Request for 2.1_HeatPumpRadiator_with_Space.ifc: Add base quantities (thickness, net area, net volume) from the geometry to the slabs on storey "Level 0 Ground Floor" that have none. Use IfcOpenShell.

First a look at what the model holds.

```python
import ifcopenshell
import ifcopenshell.util.element
import ifcopenshell.util.unit

model = ifcopenshell.open("2.1_HeatPumpRadiator_with_Space.ifc")
print(model.schema)
for unit_type in ("LENGTHUNIT", "AREAUNIT", "VOLUMEUNIT"):
    print(unit_type, ifcopenshell.util.unit.calculate_unit_scale(model, unit_type))
storey = next(s for s in model.by_type("IfcBuildingStorey") if s.Name == "Level 0 Ground Floor")
slabs = [e for e in ifcopenshell.util.element.get_decomposition(storey) if e.is_a("IfcSlab")]
for e in sorted(slabs, key=lambda e: e.id()):
    print(e.id(), e.is_a(), e.Name, list(ifcopenshell.util.element.get_psets(e, qtos_only=True)), sep=" | ")
```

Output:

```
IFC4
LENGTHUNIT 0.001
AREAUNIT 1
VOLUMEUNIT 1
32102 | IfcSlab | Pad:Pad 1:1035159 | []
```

```python
import ifcopenshell
import ifcopenshell.api.pset
import ifcopenshell.geom
import ifcopenshell.util.element
import ifcopenshell.util.shape
import ifcopenshell.util.unit

model = ifcopenshell.open("2.1_HeatPumpRadiator_with_Space.ifc")
unit_scale = ifcopenshell.util.unit.calculate_unit_scale(model)
area_scale = ifcopenshell.util.unit.calculate_unit_scale(model, "AREAUNIT")
volume_scale = ifcopenshell.util.unit.calculate_unit_scale(model, "VOLUMEUNIT")
settings = ifcopenshell.geom.settings()

storey = next(s for s in model.by_type("IfcBuildingStorey") if s.Name == "Level 0 Ground Floor")
slabs = [e for e in ifcopenshell.util.element.get_decomposition(storey) if e.is_a("IfcSlab")]

for e in sorted(slabs, key=lambda e: e.id()):
    if ifcopenshell.util.element.get_psets(e, qtos_only=True, should_inherit=False):
        continue
    # Geometry comes back in metres, in the element's own axes.
    shape = ifcopenshell.geom.create_shape(settings, e)
    values = {
        "Width": ifcopenshell.util.shape.get_z(shape.geometry) / unit_scale,
        "NetArea": ifcopenshell.util.shape.get_footprint_area(shape.geometry) / area_scale,
        "NetVolume": ifcopenshell.util.shape.get_volume(shape.geometry) / volume_scale,
    }
    qto = ifcopenshell.api.pset.add_qto(model, product=e, name="Qto_SlabBaseQuantities")
    ifcopenshell.api.pset.edit_qto(model, qto=qto, properties=values)
    print(e.id(), {k: round(v, 3) for k, v in values.items()})

model.write("2.1_HeatPumpRadiator_with_Space_v2.ifc")
```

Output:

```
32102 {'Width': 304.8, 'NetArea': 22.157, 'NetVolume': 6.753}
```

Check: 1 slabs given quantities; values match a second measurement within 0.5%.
